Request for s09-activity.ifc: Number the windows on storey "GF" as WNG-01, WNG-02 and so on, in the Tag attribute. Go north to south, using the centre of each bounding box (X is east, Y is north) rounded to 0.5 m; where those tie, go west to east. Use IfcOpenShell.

First a look at what the model holds.

```python
import ifcopenshell
import ifcopenshell.util.element
import ifcopenshell.util.placement

model = ifcopenshell.open("s09-activity.ifc")
print(model.schema)
storey = next(s for s in model.by_type("IfcBuildingStorey") if s.Name == "GF")
windows = [e for e in ifcopenshell.util.element.get_decomposition(storey) if e.is_a("IfcWindow")]
for e in sorted(windows, key=lambda e: e.id()):
    origin = ifcopenshell.util.placement.get_local_placement(e.ObjectPlacement)[:3, 3]
    print(e.id(), e.Tag, e.Name, origin.round(2) + 0.0, sep=" | ")
```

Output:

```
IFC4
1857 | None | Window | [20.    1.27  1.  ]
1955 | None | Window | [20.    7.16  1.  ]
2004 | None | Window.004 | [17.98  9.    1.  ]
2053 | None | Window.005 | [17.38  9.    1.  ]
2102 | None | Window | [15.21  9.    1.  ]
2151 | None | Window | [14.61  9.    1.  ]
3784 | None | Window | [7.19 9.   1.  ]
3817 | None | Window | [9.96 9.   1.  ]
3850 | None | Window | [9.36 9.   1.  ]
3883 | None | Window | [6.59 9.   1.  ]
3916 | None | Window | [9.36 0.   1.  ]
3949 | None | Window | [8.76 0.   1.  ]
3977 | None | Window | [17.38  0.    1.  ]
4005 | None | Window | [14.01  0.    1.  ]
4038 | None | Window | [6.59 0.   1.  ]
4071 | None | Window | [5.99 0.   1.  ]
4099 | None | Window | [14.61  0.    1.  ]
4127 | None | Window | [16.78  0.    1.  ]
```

```python
import ifcopenshell
import ifcopenshell.geom
import ifcopenshell.util.element
import ifcopenshell.util.shape

model = ifcopenshell.open("s09-activity.ifc")
settings = ifcopenshell.geom.settings()
settings.set("use-world-coords", True)


def centre(element):
    shape = ifcopenshell.geom.create_shape(settings, element)
    return ifcopenshell.util.shape.get_bbox_centroid(shape.geometry)


storey = next(s for s in model.by_type("IfcBuildingStorey") if s.Name == "GF")
windows = [e for e in ifcopenshell.util.element.get_decomposition(storey) if e.is_a("IfcWindow")]

# Insertion points can sit at a corner or the storey origin, so sort by the geometry (in metres).
centres = {e: centre(e) for e in windows}
windows.sort(key=lambda e: (-round(centres[e][1] / 0.5), centres[e][0]))

for i, e in enumerate(windows, start=1):
    number = f"WNG-{i:02d}"
    e.Tag = number
    print(e.id(), number)

model.write("s09-activity-out.ifc")
```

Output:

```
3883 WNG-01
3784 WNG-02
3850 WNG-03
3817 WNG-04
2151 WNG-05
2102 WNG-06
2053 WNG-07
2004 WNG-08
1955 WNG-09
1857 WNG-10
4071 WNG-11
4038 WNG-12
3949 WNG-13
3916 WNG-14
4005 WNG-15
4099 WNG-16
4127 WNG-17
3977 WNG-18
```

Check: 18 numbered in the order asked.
